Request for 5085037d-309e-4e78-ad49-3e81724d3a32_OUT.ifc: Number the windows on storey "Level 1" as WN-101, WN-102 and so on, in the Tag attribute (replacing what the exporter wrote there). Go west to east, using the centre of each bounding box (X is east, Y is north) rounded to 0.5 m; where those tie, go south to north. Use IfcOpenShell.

First a look at what the model holds.

```python
import ifcopenshell
import ifcopenshell.util.element
import ifcopenshell.util.placement

model = ifcopenshell.open("5085037d-309e-4e78-ad49-3e81724d3a32_OUT.ifc")
print(model.schema)
storey = next(s for s in model.by_type("IfcBuildingStorey") if s.Name == "Level 1")
windows = [e for e in ifcopenshell.util.element.get_decomposition(storey) if e.is_a("IfcWindow")]
for e in sorted(windows, key=lambda e: e.id()):
    origin = ifcopenshell.util.placement.get_local_placement(e.ObjectPlacement)[:3, 3]
    print(e.id(), e.Tag, e.Name, origin.round(2) + 0.0, sep=" | ")
```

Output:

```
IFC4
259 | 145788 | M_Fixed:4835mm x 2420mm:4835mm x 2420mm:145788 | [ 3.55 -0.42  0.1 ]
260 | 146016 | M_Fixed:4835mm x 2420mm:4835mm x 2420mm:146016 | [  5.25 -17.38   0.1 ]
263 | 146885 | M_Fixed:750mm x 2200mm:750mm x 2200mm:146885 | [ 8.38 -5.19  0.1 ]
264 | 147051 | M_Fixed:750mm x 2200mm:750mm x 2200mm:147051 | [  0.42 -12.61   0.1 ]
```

```python
import ifcopenshell
import ifcopenshell.geom
import ifcopenshell.util.element
import ifcopenshell.util.shape

model = ifcopenshell.open("5085037d-309e-4e78-ad49-3e81724d3a32_OUT.ifc")
settings = ifcopenshell.geom.settings()
settings.set("use-world-coords", True)


def centre(element):
    shape = ifcopenshell.geom.create_shape(settings, element)
    return ifcopenshell.util.shape.get_bbox_centroid(shape.geometry)


storey = next(s for s in model.by_type("IfcBuildingStorey") if s.Name == "Level 1")
windows = [e for e in ifcopenshell.util.element.get_decomposition(storey) if e.is_a("IfcWindow")]

# Insertion points can sit at a corner or the storey origin, so sort by the geometry (in metres).
centres = {e: centre(e) for e in windows}
windows.sort(key=lambda e: (round(centres[e][0] / 0.5), centres[e][1]))

for i, e in enumerate(windows, start=1):
    number = f"WN-1{i:02d}"
    e.Tag = number
    print(e.id(), number)

model.write("5085037d-309e-4e78-ad49-3e81724d3a32_OUT_rev.ifc")
```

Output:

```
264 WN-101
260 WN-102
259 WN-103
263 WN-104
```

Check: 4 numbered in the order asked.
